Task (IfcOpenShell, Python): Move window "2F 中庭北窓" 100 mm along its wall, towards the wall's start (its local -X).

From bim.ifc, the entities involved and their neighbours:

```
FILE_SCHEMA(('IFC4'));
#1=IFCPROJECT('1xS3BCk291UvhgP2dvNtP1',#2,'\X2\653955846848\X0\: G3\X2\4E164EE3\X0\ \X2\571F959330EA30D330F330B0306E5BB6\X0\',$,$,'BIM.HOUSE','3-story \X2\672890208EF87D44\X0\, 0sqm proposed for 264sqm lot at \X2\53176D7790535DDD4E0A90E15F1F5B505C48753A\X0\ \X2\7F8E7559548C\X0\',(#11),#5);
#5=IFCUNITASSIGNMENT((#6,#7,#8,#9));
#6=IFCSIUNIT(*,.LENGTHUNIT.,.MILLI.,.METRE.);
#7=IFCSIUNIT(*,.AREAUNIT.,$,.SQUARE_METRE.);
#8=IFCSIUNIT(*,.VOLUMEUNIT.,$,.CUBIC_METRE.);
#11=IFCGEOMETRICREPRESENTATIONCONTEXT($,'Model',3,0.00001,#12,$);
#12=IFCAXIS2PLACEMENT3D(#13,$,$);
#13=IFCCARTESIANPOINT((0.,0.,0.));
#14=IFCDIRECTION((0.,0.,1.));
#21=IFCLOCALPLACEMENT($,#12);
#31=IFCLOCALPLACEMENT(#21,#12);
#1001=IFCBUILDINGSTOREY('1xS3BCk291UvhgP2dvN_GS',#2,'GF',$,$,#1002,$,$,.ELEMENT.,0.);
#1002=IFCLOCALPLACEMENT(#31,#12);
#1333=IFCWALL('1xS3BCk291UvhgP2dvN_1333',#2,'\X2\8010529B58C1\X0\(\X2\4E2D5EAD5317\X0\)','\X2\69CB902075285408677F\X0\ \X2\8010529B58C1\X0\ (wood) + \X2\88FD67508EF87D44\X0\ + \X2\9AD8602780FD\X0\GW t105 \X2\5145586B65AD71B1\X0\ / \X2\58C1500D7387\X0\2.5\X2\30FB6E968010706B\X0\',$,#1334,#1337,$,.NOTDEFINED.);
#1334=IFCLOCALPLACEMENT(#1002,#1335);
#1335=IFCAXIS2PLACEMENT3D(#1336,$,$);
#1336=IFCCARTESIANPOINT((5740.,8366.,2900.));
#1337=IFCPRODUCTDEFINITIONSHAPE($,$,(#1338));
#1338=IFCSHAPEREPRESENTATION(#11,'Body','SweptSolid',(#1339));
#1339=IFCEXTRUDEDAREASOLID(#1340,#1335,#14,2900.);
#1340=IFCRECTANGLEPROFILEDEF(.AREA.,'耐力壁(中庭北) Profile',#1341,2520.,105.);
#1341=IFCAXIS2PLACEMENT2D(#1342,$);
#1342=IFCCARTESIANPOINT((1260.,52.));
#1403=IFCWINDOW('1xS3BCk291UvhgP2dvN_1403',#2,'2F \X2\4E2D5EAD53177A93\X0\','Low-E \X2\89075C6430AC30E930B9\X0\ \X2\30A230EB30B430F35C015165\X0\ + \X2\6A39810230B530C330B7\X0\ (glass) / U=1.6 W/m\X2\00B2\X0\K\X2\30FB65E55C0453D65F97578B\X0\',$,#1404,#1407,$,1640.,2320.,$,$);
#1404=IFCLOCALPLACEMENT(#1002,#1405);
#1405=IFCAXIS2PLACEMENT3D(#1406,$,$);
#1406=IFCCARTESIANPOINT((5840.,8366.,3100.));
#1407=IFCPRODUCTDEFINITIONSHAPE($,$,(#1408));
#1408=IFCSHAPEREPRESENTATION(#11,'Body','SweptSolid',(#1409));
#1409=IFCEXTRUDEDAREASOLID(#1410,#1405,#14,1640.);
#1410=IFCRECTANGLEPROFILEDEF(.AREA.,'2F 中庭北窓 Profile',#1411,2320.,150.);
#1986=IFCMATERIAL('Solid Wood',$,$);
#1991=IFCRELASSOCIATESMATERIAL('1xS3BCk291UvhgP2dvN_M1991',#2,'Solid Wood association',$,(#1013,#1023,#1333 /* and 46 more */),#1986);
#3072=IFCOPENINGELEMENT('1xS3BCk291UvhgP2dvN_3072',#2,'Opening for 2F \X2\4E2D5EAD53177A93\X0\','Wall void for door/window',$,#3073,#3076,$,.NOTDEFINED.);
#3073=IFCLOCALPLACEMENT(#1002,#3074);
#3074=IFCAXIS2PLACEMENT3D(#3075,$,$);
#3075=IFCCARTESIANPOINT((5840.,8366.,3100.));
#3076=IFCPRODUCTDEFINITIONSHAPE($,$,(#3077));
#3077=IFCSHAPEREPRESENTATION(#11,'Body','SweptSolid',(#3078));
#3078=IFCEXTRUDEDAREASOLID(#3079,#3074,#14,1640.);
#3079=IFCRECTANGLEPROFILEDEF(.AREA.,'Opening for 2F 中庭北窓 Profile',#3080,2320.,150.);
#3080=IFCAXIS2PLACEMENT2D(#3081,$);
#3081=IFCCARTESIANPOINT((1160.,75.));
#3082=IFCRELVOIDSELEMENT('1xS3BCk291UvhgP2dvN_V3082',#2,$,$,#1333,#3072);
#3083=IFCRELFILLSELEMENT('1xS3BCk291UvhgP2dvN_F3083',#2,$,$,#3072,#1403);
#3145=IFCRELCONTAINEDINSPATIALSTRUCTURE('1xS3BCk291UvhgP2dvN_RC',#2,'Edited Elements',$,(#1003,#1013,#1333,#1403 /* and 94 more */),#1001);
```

```python
import ifcopenshell
import ifcopenshell.api.geometry
import ifcopenshell.util.placement
import ifcopenshell.util.unit

model = ifcopenshell.open("bim.ifc")
unit_scale = ifcopenshell.util.unit.calculate_unit_scale(model)

window = model.by_guid("1xS3BCk291UvhgP2dvN_1403")
opening = window.FillsVoids[0].RelatingOpeningElement
wall = opening.VoidsElements[0].RelatingBuildingElement

wall_matrix = ifcopenshell.util.placement.get_local_placement(wall.ObjectPlacement)
shift = wall_matrix[:3, 0] * -0.1 / unit_scale
before = ifcopenshell.util.placement.get_local_placement(window.ObjectPlacement)[:3, 3].copy()

# The window is not placed relative to its opening, so move both.
for product in (opening, window):
    matrix = ifcopenshell.util.placement.get_local_placement(product.ObjectPlacement)
    matrix[:3, 3] += shift
    ifcopenshell.api.geometry.edit_object_placement(model, product=product, matrix=matrix, is_si=False)

after = ifcopenshell.util.placement.get_local_placement(window.ObjectPlacement)[:3, 3]
print("window moved by", (after - before).round(3) + 0.0)

model.write("bim_rev.ifc")
```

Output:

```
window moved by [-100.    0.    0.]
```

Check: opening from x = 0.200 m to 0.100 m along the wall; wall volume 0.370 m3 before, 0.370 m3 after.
